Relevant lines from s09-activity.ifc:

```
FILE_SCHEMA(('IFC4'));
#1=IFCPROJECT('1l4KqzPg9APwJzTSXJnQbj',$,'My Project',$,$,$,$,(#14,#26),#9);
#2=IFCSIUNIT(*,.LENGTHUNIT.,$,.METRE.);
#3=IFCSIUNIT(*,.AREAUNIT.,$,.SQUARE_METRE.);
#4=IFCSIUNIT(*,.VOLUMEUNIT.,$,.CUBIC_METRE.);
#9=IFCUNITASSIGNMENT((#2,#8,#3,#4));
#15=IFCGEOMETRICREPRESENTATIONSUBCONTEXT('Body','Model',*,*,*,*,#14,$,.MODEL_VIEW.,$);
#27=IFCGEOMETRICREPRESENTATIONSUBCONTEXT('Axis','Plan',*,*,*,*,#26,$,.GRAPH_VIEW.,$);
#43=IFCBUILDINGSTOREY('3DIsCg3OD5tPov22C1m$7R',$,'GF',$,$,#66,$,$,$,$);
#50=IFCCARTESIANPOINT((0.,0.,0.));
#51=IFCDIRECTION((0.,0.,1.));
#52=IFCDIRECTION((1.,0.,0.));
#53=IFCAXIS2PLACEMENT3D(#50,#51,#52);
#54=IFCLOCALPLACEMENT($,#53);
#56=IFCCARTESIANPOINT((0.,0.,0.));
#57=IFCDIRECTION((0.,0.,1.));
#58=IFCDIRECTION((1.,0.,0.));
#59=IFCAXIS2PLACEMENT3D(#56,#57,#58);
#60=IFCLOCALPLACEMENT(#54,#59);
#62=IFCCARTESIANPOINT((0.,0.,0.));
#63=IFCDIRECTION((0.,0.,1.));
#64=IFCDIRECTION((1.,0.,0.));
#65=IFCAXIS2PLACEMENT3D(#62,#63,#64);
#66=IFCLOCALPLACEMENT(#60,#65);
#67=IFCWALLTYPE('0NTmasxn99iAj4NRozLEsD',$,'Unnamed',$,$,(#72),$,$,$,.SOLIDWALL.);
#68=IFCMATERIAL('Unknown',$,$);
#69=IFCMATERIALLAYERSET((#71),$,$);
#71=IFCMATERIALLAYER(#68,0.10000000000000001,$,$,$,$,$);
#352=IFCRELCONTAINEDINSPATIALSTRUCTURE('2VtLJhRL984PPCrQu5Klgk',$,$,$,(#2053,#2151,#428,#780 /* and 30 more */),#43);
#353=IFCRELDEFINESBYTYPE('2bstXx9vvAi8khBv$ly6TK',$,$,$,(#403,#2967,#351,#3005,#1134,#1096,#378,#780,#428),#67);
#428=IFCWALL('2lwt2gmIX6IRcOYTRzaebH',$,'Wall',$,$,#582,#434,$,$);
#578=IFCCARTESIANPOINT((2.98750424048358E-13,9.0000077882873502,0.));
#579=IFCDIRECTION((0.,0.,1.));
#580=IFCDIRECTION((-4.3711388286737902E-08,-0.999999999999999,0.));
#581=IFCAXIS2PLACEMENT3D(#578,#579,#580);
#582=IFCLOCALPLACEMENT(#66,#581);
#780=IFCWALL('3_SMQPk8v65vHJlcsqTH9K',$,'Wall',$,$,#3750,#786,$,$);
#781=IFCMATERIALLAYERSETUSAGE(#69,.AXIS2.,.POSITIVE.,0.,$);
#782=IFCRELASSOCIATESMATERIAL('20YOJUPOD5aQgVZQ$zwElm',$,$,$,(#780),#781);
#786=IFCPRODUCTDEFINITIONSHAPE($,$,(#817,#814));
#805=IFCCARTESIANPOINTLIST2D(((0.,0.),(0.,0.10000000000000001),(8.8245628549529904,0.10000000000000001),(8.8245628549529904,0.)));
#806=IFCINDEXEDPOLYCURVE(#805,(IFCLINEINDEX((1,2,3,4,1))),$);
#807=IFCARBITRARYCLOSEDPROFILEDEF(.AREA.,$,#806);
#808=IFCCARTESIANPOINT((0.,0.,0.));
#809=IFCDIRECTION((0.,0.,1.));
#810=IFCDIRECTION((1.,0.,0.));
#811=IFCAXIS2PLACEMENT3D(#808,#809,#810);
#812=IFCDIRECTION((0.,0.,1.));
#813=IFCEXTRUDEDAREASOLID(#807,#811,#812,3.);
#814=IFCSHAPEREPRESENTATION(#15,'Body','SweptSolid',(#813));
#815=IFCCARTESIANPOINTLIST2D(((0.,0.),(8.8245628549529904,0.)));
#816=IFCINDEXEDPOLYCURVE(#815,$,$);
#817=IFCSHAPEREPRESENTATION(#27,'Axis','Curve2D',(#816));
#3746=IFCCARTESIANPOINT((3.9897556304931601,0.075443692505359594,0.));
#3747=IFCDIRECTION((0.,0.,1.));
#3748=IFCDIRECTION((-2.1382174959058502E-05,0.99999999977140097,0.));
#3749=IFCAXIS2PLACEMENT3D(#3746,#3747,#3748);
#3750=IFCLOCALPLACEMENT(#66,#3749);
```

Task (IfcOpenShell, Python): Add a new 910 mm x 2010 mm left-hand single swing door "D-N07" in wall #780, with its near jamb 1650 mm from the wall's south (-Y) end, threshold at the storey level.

```python
import numpy as np
import ifcopenshell
import ifcopenshell.api.feature
import ifcopenshell.api.geometry
import ifcopenshell.api.root
import ifcopenshell.api.spatial
import ifcopenshell.geom
import ifcopenshell.util.element
import ifcopenshell.util.placement
import ifcopenshell.util.representation
import ifcopenshell.util.shape
import ifcopenshell.util.unit

model = ifcopenshell.open("s09-activity.ifc")
unit_scale = ifcopenshell.util.unit.calculate_unit_scale(model)
settings = ifcopenshell.geom.settings()


def volume(element):
    """Net volume in cubic metres, openings subtracted."""
    shape = ifcopenshell.geom.create_shape(settings, element)
    return ifcopenshell.util.shape.get_volume(shape.geometry)


wall = model.by_id(780)
storey = ifcopenshell.util.element.get_container(wall, ifc_class="IfcBuildingStorey")
context = ifcopenshell.util.representation.get_context(model, "Model", "Body", "MODEL_VIEW")
before = volume(wall)

width, height, from_end, sill = 0.91, 2.01, 1.65, 0.0  # metres

# The wall runs along its own X axis, and the end named is its -X end.
wall_shape = ifcopenshell.geom.create_shape(settings, wall)
x, y, z = ifcopenshell.util.shape.get_vertices(wall_shape.geometry).T
start = x.min() + from_end
face, thickness = float(y.min()), float(y.max() - y.min())
wall_matrix = ifcopenshell.util.placement.get_local_placement(wall.ObjectPlacement)
level = ifcopenshell.util.placement.get_local_placement(storey.ObjectPlacement)[2, 3]


def in_wall(x, y):
    """Placement at x, y metres in the wall's axes, at sill height."""
    matrix = wall_matrix.copy()
    matrix[:, 3] = wall_matrix @ np.array([x / unit_scale, y / unit_scale, 0.0, 1.0])
    matrix[2, 3] = level + sill / unit_scale
    return matrix


# Opening: a box that overshoots both wall faces by 50 mm.
opening = ifcopenshell.api.root.create_entity(model, ifc_class="IfcOpeningElement", predefined_type="OPENING")
box = ifcopenshell.api.geometry.add_wall_representation(
    model, context=context, length=width, height=height, thickness=thickness + 0.1
)
ifcopenshell.api.geometry.assign_representation(model, product=opening, representation=box)
ifcopenshell.api.geometry.edit_object_placement(model, product=opening, matrix=in_wall(start, face - 0.05), is_si=False)
ifcopenshell.api.feature.add_feature(model, feature=opening, element=wall)

door = ifcopenshell.api.root.create_entity(model, ifc_class="IfcDoor", name="D-N07", predefined_type="DOOR")
door.OverallWidth, door.OverallHeight = width / unit_scale, height / unit_scale
door.OperationType = "SINGLE_SWING_LEFT"
body = ifcopenshell.api.geometry.add_door_representation(
    model,
    context=context,
    overall_width=door.OverallWidth,
    overall_height=door.OverallHeight,
    operation_type="SINGLE_SWING_LEFT",
    lining_properties={"LiningDepth": thickness / unit_scale, "ThresholdDepth": thickness / unit_scale},
)
ifcopenshell.api.geometry.assign_representation(model, product=door, representation=body)
ifcopenshell.api.spatial.assign_container(model, products=[door], relating_structure=storey)
ifcopenshell.api.feature.add_filling(model, opening=opening, element=door)

# The lining spans the wall, so the door starts at the wall face.
ifcopenshell.api.geometry.edit_object_placement(model, product=door, matrix=in_wall(start, face), is_si=False)

after = volume(wall)

print(f"wall volume {before:.3f} -> {after:.3f} m3")

model.write("s09-activity-out.ifc")
```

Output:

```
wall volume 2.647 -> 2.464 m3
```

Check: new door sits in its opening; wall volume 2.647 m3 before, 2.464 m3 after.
